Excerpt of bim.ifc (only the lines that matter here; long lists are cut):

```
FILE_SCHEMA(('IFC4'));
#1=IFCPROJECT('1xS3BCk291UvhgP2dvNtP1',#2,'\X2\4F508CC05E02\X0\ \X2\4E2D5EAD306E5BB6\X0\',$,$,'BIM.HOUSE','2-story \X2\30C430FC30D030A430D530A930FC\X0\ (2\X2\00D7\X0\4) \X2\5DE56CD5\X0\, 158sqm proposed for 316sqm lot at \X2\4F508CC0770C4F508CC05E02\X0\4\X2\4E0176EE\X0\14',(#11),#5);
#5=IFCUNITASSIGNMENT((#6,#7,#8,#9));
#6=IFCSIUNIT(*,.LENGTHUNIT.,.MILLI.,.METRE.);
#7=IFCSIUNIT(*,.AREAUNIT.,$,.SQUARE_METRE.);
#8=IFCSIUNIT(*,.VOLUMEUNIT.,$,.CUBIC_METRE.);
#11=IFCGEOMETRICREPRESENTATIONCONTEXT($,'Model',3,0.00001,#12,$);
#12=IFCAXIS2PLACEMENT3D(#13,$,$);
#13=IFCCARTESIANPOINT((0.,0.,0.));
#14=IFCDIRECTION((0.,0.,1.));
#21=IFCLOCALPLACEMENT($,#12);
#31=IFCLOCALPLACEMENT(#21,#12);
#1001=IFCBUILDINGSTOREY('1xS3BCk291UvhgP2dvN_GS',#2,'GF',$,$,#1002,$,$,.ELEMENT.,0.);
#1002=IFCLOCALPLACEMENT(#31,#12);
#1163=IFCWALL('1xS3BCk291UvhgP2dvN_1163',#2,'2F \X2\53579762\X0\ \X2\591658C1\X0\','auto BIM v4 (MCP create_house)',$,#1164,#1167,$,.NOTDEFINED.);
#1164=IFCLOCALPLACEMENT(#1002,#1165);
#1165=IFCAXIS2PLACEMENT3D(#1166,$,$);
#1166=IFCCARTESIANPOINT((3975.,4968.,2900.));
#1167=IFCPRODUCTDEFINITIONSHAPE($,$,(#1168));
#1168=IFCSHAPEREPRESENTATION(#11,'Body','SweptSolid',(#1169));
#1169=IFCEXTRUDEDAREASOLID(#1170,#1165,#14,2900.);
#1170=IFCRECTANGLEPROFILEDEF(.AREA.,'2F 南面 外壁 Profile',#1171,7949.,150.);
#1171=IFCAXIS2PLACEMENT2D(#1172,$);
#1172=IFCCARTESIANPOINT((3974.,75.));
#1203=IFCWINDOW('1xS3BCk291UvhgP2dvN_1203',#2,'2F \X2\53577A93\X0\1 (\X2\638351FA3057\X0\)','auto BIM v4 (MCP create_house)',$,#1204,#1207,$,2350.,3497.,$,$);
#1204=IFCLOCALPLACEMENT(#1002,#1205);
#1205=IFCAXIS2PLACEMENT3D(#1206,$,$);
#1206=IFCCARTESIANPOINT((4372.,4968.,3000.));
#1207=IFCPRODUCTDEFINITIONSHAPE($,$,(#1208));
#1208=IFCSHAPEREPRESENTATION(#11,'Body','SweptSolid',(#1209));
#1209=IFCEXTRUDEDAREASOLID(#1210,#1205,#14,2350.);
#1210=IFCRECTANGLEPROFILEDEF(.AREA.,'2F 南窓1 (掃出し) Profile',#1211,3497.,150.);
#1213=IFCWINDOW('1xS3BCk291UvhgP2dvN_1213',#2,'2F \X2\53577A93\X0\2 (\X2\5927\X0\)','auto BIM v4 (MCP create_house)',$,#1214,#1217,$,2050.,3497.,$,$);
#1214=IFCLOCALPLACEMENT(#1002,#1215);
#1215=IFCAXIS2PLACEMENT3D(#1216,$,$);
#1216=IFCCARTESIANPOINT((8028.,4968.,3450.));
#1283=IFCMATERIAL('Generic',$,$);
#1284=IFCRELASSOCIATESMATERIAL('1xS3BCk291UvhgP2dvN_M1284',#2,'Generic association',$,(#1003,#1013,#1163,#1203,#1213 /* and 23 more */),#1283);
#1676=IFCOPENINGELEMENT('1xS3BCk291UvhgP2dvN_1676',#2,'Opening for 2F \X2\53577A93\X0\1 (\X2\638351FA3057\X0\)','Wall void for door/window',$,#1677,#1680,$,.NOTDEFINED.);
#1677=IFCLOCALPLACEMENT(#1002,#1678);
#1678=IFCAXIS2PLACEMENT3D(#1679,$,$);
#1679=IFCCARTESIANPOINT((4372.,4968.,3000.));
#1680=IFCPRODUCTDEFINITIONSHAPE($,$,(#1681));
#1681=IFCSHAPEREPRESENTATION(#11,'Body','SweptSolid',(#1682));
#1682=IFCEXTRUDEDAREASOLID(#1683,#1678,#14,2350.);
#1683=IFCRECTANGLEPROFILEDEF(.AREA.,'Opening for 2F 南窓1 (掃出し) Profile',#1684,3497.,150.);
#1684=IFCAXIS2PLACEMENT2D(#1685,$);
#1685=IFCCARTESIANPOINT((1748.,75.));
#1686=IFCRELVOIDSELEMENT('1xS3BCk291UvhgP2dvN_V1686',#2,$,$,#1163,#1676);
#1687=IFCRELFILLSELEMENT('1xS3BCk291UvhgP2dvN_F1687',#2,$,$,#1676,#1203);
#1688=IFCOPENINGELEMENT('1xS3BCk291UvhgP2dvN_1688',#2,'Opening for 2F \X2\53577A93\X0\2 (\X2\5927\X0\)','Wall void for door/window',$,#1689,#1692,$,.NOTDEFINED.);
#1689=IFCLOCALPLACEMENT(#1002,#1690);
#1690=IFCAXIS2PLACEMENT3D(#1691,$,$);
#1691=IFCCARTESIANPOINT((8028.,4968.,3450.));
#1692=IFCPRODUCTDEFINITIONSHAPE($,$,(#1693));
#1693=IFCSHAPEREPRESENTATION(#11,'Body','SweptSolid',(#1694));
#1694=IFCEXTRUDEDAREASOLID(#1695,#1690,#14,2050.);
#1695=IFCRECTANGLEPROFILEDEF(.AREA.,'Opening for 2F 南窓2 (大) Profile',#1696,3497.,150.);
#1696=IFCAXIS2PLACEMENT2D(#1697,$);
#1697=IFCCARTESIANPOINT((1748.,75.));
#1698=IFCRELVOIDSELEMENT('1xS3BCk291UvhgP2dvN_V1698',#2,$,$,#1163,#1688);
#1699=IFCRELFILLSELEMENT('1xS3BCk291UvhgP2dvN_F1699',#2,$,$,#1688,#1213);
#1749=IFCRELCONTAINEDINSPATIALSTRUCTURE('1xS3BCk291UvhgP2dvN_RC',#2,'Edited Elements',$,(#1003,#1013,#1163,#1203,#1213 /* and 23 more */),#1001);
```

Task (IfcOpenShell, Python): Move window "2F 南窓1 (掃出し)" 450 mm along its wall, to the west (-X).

```python
import ifcopenshell
import ifcopenshell.api.geometry
import ifcopenshell.util.placement

model = ifcopenshell.open("bim.ifc")

window = model.by_id(1203)
opening = window.FillsVoids[0].RelatingOpeningElement
wall = opening.VoidsElements[0].RelatingBuildingElement

wall_matrix = ifcopenshell.util.placement.get_local_placement(wall.ObjectPlacement)
shift = wall_matrix[:3, 0] * -450.0
before = ifcopenshell.util.placement.get_local_placement(window.ObjectPlacement)[:3, 3].copy()

# The window is not placed relative to its opening, so move both.
for product in (opening, window):
    matrix = ifcopenshell.util.placement.get_local_placement(product.ObjectPlacement)
    matrix[:3, 3] += shift
    ifcopenshell.api.geometry.edit_object_placement(model, product=product, matrix=matrix, is_si=False)

after = ifcopenshell.util.placement.get_local_placement(window.ObjectPlacement)[:3, 3]
print("window moved by", (after - before).round(3) + 0.0)

model.write("bim_edited.ifc")
```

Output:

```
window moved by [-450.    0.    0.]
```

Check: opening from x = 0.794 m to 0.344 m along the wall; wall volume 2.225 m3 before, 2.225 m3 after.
